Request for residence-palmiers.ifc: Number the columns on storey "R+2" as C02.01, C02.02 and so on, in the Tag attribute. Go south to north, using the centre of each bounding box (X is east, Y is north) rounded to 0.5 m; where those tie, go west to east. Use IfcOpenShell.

First a look at what the model holds.

```python
import ifcopenshell
import ifcopenshell.util.element
import ifcopenshell.util.placement

model = ifcopenshell.open("residence-palmiers.ifc")
print(model.schema)
storey = next(s for s in model.by_type("IfcBuildingStorey") if s.Name == "R+2")
columns = [e for e in ifcopenshell.util.element.get_decomposition(storey) if e.is_a("IfcColumn")]
for e in sorted(columns, key=lambda e: e.id()):
    origin = ifcopenshell.util.placement.get_local_placement(e.ObjectPlacement)[:3, 3]
    print(e.id(), e.Tag, e.Name, origin.round(2) + 0.0, sep=" | ")
```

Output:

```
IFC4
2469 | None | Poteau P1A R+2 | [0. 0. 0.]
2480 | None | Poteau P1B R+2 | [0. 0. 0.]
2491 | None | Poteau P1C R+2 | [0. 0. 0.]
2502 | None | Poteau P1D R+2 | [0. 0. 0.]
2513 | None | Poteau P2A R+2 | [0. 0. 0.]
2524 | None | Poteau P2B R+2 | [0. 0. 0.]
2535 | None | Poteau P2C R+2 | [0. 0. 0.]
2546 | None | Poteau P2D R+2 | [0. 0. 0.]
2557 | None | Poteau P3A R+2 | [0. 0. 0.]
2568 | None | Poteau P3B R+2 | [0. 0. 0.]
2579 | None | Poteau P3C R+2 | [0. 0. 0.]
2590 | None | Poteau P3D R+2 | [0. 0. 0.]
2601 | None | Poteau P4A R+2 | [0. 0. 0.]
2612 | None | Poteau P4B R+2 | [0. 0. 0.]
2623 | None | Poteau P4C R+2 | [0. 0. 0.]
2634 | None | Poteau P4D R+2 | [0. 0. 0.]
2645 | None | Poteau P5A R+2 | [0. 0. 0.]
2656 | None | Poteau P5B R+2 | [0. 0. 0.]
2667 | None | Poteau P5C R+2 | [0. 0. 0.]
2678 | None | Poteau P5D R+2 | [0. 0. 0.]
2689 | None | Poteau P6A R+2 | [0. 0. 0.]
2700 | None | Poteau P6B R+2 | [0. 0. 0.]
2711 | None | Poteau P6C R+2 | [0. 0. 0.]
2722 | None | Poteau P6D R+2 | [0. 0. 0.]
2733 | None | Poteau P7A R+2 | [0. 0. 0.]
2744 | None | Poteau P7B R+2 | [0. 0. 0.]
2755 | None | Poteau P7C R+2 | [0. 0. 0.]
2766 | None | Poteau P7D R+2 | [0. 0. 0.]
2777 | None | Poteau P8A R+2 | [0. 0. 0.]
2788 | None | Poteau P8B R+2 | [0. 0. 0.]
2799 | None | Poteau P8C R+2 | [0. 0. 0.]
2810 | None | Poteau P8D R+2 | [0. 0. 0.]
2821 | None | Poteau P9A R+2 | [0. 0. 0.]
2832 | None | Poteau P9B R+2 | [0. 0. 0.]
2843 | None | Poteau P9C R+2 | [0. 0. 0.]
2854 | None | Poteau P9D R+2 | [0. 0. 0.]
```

```python
import ifcopenshell
import ifcopenshell.geom
import ifcopenshell.util.element
import ifcopenshell.util.shape

model = ifcopenshell.open("residence-palmiers.ifc")
settings = ifcopenshell.geom.settings()
settings.set("use-world-coords", True)


def centre(element):
    shape = ifcopenshell.geom.create_shape(settings, element)
    return ifcopenshell.util.shape.get_bbox_centroid(shape.geometry)


storey = next(s for s in model.by_type("IfcBuildingStorey") if s.Name == "R+2")
columns = [e for e in ifcopenshell.util.element.get_decomposition(storey) if e.is_a("IfcColumn")]

# Insertion points can sit at a corner or the storey origin, so sort by the geometry (in metres).
centres = {e: centre(e) for e in columns}
columns.sort(key=lambda e: (round(centres[e][1] / 0.5), centres[e][0]))

for i, e in enumerate(columns, start=1):
    number = f"C02.{i:02d}"
    e.Tag = number
    print(e.id(), number)

model.write("residence-palmiers-out.ifc")
```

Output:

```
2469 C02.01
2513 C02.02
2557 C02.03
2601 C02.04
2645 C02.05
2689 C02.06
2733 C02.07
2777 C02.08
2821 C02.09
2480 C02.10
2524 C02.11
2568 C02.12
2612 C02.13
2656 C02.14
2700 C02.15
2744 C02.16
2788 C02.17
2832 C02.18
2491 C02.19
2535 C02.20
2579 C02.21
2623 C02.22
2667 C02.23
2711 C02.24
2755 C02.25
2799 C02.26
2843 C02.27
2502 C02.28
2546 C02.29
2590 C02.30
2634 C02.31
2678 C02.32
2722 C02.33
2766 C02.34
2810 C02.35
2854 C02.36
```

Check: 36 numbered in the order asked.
